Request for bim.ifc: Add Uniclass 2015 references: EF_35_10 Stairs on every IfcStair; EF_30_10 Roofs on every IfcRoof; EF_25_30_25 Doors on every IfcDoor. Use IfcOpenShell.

First a look at what the model holds.

```python
import ifcopenshell

model = ifcopenshell.open("bim.ifc")
print(model.schema)
print("classifications:", [c.Name for c in model.by_type("IfcClassification")])
for ifc_class in ("IfcDoor", "IfcRoof", "IfcStair", "IfcWall", "IfcWindow"):
    print(ifc_class, len(model.by_type(ifc_class)))
```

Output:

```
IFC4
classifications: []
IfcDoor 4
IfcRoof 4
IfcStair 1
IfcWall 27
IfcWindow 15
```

```python
import ifcopenshell
import ifcopenshell.api.classification

model = ifcopenshell.open("bim.ifc")

system = ifcopenshell.api.classification.add_classification(model, classification="Uniclass 2015")

codes = {
    "IfcStair": ("EF_35_10", "Stairs"),
    "IfcRoof": ("EF_30_10", "Roofs"),
    "IfcDoor": ("EF_25_30_25", "Doors"),
}
for ifc_class, (code, name) in codes.items():
    products = model.by_type(ifc_class)
    ifcopenshell.api.classification.add_reference(
        model, products=products, classification=system, identification=code, name=name
    )
    print(code, len(products))

model.write("bim_v2.ifc")
```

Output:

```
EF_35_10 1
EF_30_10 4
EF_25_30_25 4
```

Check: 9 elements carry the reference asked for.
